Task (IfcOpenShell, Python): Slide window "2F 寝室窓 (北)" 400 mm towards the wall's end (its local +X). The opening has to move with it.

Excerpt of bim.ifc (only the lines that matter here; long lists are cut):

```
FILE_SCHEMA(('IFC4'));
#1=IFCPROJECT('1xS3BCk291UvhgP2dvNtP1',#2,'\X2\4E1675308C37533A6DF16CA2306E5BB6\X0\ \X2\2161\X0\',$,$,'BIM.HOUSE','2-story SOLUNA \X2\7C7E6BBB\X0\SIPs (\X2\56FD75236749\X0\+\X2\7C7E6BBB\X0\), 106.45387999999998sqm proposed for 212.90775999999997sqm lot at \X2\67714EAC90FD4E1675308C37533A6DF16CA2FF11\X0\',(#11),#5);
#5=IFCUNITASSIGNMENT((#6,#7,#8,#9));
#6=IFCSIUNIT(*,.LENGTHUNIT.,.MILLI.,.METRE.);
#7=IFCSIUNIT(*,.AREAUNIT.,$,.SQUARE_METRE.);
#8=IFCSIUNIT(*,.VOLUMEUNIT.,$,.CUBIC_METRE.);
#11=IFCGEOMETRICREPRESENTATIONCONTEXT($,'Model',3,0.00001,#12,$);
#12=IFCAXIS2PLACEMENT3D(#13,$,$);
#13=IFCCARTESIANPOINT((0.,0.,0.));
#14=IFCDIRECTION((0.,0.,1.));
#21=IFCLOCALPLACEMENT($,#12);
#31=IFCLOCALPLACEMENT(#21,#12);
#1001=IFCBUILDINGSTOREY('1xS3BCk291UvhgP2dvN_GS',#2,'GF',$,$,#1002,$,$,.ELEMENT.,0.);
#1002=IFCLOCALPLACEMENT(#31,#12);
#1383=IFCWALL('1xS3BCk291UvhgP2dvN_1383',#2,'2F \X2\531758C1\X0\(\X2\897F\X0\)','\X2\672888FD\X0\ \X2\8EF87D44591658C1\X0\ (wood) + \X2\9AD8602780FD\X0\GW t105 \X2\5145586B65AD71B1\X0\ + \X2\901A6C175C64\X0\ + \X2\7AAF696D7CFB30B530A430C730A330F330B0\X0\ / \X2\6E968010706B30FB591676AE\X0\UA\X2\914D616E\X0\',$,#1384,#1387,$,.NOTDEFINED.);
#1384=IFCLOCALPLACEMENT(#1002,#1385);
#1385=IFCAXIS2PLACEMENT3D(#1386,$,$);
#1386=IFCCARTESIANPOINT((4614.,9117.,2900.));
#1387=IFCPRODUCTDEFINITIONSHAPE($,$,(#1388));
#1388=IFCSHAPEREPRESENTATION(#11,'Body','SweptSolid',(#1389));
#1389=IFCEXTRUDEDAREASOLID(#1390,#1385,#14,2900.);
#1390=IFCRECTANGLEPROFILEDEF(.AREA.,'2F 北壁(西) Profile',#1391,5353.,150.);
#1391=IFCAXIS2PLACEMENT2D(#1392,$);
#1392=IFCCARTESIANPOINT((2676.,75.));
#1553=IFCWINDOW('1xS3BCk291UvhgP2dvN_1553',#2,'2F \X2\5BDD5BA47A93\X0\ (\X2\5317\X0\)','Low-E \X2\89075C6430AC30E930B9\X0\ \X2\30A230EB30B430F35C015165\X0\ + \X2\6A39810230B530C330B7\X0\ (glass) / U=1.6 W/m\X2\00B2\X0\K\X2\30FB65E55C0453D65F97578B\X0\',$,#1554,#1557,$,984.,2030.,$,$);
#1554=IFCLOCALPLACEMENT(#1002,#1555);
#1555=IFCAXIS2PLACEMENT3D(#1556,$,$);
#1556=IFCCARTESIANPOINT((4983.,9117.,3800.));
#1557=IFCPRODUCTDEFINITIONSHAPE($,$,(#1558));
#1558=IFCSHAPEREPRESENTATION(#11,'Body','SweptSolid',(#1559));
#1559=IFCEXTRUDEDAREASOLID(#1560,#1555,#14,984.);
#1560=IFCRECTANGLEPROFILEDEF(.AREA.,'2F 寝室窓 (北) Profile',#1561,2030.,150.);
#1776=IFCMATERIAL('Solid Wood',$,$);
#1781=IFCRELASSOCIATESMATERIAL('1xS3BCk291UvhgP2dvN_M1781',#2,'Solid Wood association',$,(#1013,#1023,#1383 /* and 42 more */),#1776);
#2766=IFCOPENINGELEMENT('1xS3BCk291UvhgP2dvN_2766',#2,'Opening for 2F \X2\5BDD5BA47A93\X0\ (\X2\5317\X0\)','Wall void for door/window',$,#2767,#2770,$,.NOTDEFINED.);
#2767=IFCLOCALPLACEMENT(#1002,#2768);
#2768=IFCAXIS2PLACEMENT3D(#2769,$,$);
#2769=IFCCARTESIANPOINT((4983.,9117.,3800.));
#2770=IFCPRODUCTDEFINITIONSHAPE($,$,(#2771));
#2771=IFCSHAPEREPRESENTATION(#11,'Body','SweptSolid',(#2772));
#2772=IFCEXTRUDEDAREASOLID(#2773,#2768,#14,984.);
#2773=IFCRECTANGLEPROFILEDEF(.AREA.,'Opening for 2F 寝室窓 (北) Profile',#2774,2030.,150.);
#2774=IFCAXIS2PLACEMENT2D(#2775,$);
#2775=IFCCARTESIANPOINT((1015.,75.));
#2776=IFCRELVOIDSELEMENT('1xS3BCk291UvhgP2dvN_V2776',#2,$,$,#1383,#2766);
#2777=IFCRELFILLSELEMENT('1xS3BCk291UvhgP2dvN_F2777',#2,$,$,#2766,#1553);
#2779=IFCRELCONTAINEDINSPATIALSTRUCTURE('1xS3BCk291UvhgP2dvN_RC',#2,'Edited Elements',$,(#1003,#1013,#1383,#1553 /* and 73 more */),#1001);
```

```python
import ifcopenshell
import ifcopenshell.api.geometry
import ifcopenshell.util.placement
import ifcopenshell.util.unit

model = ifcopenshell.open("bim.ifc")
unit_scale = ifcopenshell.util.unit.calculate_unit_scale(model)

window = model.by_id(1553)
opening = window.FillsVoids[0].RelatingOpeningElement
wall = opening.VoidsElements[0].RelatingBuildingElement

wall_matrix = ifcopenshell.util.placement.get_local_placement(wall.ObjectPlacement)
shift = wall_matrix[:3, 0] * 0.4 / unit_scale
before = ifcopenshell.util.placement.get_local_placement(window.ObjectPlacement)[:3, 3].copy()

# The window is not placed relative to its opening, so move both.
for product in (opening, window):
    matrix = ifcopenshell.util.placement.get_local_placement(product.ObjectPlacement)
    matrix[:3, 3] += shift
    ifcopenshell.api.geometry.edit_object_placement(model, product=product, matrix=matrix, is_si=False)

after = ifcopenshell.util.placement.get_local_placement(window.ObjectPlacement)[:3, 3]
print("window moved by", (after - before).round(3) + 0.0)

model.write("bim_edited.ifc")
```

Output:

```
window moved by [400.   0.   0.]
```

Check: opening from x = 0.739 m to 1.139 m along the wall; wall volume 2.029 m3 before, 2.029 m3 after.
